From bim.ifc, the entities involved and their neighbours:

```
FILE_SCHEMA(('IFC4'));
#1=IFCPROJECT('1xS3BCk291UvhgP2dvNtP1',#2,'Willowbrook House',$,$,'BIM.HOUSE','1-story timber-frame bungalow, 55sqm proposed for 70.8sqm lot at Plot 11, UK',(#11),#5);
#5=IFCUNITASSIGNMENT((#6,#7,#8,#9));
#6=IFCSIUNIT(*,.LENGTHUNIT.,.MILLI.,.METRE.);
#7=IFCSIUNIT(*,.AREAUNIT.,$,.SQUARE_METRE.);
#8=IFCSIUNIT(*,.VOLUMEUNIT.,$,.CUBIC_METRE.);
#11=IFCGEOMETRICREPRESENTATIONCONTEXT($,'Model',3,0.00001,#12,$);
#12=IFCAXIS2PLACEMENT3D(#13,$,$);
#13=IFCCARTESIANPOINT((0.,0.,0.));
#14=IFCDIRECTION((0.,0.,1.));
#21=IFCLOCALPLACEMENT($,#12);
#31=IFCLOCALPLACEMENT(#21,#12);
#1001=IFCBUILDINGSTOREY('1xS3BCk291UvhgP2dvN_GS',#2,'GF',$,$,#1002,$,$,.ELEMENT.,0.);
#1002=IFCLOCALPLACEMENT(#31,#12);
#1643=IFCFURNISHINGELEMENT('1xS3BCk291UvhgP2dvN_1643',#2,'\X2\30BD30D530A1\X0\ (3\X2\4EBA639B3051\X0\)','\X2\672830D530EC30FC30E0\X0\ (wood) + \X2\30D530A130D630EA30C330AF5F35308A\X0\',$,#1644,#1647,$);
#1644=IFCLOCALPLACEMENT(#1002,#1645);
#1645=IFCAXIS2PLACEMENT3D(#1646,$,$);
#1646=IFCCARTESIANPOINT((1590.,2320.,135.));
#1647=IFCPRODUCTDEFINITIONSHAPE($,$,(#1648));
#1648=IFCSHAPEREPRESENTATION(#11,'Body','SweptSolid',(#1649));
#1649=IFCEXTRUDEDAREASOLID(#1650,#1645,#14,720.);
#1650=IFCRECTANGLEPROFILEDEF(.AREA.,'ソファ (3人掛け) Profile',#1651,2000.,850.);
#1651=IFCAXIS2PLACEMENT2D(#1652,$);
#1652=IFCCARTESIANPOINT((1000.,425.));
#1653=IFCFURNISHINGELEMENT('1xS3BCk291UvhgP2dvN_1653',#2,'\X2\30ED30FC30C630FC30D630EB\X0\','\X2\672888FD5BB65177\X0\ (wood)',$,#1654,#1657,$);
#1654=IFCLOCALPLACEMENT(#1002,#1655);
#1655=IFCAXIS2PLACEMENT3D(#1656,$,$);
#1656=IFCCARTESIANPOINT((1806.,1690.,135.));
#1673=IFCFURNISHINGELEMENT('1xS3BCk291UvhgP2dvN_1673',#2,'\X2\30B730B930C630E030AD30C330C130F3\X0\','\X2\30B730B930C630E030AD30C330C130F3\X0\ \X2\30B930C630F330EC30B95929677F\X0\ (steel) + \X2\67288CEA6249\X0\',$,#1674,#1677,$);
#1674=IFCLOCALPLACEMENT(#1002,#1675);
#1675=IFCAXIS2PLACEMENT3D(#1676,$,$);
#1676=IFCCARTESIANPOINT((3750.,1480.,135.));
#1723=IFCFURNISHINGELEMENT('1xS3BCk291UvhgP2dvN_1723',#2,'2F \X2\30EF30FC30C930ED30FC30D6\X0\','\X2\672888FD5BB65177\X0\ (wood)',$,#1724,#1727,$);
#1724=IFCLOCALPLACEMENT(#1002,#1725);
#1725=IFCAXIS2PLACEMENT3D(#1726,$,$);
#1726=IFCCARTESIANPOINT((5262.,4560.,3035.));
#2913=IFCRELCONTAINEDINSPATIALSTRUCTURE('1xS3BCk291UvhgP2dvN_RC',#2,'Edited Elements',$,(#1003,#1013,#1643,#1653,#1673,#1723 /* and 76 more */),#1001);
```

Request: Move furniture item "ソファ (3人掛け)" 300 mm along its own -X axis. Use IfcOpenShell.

```python
import ifcopenshell
import ifcopenshell.api.geometry
import ifcopenshell.util.placement
import ifcopenshell.util.unit

model = ifcopenshell.open("bim.ifc")
unit_scale = ifcopenshell.util.unit.calculate_unit_scale(model)

item = model.by_guid("1xS3BCk291UvhgP2dvN_1643")
matrix = ifcopenshell.util.placement.get_local_placement(item.ObjectPlacement)
matrix[:3, 3] -= matrix[:3, 0] * 0.3 / unit_scale
ifcopenshell.api.geometry.edit_object_placement(model, product=item, matrix=matrix, is_si=False)

print(ifcopenshell.util.placement.get_local_placement(item.ObjectPlacement).round(3) + 0.0)

model.write("bim_v2.ifc")
```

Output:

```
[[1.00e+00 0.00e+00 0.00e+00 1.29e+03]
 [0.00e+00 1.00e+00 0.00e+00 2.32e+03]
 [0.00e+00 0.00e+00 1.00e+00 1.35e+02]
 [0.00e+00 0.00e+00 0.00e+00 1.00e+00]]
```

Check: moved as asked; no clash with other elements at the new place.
